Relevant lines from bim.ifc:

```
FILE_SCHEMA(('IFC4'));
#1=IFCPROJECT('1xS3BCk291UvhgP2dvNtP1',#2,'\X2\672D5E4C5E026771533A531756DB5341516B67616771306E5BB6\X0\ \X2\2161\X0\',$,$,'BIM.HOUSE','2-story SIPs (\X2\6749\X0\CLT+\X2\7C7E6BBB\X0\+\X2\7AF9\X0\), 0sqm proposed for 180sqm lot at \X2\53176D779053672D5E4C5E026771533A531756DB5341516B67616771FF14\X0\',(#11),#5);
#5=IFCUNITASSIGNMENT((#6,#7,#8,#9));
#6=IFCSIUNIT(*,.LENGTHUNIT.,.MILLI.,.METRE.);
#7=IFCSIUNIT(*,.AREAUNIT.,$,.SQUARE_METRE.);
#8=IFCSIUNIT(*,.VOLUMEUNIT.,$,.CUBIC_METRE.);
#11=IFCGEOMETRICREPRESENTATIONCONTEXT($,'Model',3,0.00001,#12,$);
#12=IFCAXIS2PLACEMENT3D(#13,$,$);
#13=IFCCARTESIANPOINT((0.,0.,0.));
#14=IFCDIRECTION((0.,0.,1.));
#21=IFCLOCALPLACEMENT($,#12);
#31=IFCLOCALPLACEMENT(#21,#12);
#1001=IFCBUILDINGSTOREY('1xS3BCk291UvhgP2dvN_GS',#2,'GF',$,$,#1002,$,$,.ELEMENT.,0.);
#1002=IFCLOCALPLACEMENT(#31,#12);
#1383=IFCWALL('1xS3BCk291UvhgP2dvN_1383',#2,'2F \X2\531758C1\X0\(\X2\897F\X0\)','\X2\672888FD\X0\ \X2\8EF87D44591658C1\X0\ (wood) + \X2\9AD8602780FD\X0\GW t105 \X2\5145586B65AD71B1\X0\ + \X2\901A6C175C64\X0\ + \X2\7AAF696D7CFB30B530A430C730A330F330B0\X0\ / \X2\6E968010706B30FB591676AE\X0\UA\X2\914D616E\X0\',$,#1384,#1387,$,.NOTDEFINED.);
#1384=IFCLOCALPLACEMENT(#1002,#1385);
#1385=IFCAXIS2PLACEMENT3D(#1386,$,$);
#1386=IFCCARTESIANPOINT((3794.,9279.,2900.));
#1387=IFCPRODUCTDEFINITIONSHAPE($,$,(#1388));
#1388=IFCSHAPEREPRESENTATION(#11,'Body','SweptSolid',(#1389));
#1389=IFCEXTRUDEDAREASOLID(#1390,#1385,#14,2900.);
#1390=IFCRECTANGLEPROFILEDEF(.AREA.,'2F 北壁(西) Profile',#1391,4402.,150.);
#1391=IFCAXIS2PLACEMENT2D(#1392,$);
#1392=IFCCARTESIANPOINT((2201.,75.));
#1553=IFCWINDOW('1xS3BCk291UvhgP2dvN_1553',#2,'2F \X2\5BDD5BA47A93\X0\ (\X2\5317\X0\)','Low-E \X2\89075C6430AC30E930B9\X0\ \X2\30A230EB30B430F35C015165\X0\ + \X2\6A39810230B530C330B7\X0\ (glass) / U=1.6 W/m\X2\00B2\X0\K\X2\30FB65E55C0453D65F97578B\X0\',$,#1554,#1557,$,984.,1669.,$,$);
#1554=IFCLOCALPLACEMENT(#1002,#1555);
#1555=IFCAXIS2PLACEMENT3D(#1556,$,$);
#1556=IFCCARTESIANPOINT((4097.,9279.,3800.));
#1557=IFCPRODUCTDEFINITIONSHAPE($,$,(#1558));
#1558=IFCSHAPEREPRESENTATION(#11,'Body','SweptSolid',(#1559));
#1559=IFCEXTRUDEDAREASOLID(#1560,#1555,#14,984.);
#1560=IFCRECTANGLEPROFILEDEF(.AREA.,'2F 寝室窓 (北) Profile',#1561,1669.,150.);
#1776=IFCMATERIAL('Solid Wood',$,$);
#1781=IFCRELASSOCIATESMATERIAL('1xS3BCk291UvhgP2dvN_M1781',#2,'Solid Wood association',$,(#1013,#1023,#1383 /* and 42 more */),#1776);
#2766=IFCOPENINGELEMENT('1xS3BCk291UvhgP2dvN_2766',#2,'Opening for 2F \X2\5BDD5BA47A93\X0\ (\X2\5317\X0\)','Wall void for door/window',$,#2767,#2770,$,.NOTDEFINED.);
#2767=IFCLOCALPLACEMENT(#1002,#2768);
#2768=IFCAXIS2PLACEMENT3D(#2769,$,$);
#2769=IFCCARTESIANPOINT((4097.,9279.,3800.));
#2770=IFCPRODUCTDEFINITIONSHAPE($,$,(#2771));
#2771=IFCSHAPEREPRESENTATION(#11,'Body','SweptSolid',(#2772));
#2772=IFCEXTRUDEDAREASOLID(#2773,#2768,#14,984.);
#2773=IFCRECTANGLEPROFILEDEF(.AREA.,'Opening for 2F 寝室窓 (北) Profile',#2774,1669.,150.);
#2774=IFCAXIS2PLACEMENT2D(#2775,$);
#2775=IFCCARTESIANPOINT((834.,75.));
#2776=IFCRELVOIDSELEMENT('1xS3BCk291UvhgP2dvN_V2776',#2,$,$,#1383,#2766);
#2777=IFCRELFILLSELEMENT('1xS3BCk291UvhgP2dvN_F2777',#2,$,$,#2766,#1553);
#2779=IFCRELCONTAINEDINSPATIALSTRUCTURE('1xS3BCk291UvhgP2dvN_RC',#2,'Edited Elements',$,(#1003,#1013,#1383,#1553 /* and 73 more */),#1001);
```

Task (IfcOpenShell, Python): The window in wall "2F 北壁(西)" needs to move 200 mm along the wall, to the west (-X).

```python
import ifcopenshell
import ifcopenshell.api.geometry
import ifcopenshell.util.placement

model = ifcopenshell.open("bim.ifc")

window = model.by_id(1553)
opening = window.FillsVoids[0].RelatingOpeningElement
wall = opening.VoidsElements[0].RelatingBuildingElement

wall_matrix = ifcopenshell.util.placement.get_local_placement(wall.ObjectPlacement)
shift = wall_matrix[:3, 0] * -200.0
before = ifcopenshell.util.placement.get_local_placement(window.ObjectPlacement)[:3, 3].copy()

# The window is not placed relative to its opening, so move both.
for product in (opening, window):
    matrix = ifcopenshell.util.placement.get_local_placement(product.ObjectPlacement)
    matrix[:3, 3] += shift
    ifcopenshell.api.geometry.edit_object_placement(model, product=product, matrix=matrix, is_si=False)

after = ifcopenshell.util.placement.get_local_placement(window.ObjectPlacement)[:3, 3]
print("window moved by", (after - before).round(3) + 0.0)

model.write("bim_updated.ifc")
```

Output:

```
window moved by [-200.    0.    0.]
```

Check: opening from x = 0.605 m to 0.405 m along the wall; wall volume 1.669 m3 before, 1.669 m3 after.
